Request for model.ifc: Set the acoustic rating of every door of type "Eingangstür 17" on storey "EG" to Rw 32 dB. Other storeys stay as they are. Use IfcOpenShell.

First a look at what the model holds.

```python
import ifcopenshell
import ifcopenshell.util.element

model = ifcopenshell.open("model.ifc")
print(model.schema)
storey = next(s for s in model.by_type("IfcBuildingStorey") if s.Name == "EG")
doors = [e for e in ifcopenshell.util.element.get_decomposition(storey) if e.is_a("IfcDoor")]
seen = {}
for e in doors:
    element_type = ifcopenshell.util.element.get_type(e)
    key = (element_type.Name if element_type != e and element_type else None, ifcopenshell.util.element.get_pset(e, "Pset_DoorCommon", "AcousticRating"))
    seen[key] = seen.get(key, 0) + 1
for (name, value), count in sorted(seen.items(), key=str):
    print(count, "x", name, "|", value)
```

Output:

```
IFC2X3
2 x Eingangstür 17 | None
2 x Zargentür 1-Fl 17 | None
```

```python
import ifcopenshell
import ifcopenshell.api.pset
import ifcopenshell.util.element

model = ifcopenshell.open("model.ifc")

storey = next(s for s in model.by_type("IfcBuildingStorey") if s.Name == "EG")
doors = [e for e in ifcopenshell.util.element.get_decomposition(storey) if e.is_a("IfcDoor")]

count = 0
for e in doors:
    element_type = ifcopenshell.util.element.get_type(e)
    if element_type in (None, e) or element_type.Name != "Eingangstür 17":
        continue
    # add_pset returns the element's existing set when there is one.
    pset = ifcopenshell.api.pset.add_pset(model, product=e, name="Pset_DoorCommon")
    ifcopenshell.api.pset.edit_pset(model, pset=pset, properties={"AcousticRating": "Rw 32 dB"})
    count += 1

print(count, "doors updated")

model.write("model_v2.ifc")
```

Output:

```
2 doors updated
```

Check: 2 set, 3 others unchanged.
